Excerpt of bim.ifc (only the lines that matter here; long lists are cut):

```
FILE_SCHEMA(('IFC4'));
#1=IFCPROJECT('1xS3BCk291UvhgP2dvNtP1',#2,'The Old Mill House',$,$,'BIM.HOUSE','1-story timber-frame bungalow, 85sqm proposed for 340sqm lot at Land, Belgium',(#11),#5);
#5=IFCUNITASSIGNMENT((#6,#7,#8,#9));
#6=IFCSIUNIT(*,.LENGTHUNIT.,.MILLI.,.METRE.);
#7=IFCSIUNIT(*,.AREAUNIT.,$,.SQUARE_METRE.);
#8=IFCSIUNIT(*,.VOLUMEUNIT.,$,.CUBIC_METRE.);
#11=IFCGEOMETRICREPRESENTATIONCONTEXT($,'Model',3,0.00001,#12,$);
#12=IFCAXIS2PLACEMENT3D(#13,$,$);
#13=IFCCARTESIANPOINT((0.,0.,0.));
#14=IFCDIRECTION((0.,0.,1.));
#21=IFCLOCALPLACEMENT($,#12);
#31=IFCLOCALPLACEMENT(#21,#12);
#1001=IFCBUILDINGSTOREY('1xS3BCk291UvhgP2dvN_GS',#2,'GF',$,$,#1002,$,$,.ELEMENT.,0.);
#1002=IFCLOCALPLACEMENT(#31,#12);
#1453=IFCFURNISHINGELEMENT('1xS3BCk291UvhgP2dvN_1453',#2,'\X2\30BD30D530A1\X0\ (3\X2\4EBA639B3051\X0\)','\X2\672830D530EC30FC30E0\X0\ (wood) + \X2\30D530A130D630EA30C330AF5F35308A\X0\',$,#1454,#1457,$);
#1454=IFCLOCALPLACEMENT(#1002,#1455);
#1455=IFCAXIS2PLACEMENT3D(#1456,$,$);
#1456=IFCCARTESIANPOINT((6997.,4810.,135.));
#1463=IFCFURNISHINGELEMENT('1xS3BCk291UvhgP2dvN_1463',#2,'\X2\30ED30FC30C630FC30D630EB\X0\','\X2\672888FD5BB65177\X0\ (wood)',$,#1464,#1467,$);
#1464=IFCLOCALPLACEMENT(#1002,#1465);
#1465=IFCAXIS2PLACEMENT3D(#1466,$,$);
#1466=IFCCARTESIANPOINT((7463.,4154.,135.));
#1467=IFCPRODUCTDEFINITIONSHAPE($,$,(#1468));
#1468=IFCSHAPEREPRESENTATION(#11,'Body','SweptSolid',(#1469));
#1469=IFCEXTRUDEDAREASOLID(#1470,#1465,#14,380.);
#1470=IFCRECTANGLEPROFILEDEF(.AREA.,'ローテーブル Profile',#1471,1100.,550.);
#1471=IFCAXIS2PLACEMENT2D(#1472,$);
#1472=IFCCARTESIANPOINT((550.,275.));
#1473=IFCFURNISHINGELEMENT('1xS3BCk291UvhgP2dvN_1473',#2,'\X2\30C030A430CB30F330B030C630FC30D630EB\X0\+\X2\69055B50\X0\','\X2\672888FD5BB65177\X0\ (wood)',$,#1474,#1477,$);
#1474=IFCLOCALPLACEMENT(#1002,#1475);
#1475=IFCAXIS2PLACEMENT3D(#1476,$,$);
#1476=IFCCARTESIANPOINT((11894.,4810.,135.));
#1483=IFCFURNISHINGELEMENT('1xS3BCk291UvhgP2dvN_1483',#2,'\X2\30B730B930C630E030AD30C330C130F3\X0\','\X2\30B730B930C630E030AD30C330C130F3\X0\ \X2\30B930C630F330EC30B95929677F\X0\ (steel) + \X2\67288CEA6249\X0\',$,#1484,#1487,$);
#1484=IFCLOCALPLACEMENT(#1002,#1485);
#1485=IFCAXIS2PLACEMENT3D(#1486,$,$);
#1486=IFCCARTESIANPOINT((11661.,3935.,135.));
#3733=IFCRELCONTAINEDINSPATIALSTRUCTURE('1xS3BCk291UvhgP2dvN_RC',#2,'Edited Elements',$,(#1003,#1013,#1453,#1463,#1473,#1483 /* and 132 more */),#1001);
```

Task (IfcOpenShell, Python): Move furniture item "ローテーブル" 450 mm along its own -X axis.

```python
import ifcopenshell
import ifcopenshell.api.geometry
import ifcopenshell.util.placement
import ifcopenshell.util.unit

model = ifcopenshell.open("bim.ifc")
unit_scale = ifcopenshell.util.unit.calculate_unit_scale(model)

item = model.by_guid("1xS3BCk291UvhgP2dvN_1463")
matrix = ifcopenshell.util.placement.get_local_placement(item.ObjectPlacement)
matrix[:3, 3] -= matrix[:3, 0] * 0.45 / unit_scale
ifcopenshell.api.geometry.edit_object_placement(model, product=item, matrix=matrix, is_si=False)

print(ifcopenshell.util.placement.get_local_placement(item.ObjectPlacement).round(3) + 0.0)

model.write("bim_v2.ifc")
```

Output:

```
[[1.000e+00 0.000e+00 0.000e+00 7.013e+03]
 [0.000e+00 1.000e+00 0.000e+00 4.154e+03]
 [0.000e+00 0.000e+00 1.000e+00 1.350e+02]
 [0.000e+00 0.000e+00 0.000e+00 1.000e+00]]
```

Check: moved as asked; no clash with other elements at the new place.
